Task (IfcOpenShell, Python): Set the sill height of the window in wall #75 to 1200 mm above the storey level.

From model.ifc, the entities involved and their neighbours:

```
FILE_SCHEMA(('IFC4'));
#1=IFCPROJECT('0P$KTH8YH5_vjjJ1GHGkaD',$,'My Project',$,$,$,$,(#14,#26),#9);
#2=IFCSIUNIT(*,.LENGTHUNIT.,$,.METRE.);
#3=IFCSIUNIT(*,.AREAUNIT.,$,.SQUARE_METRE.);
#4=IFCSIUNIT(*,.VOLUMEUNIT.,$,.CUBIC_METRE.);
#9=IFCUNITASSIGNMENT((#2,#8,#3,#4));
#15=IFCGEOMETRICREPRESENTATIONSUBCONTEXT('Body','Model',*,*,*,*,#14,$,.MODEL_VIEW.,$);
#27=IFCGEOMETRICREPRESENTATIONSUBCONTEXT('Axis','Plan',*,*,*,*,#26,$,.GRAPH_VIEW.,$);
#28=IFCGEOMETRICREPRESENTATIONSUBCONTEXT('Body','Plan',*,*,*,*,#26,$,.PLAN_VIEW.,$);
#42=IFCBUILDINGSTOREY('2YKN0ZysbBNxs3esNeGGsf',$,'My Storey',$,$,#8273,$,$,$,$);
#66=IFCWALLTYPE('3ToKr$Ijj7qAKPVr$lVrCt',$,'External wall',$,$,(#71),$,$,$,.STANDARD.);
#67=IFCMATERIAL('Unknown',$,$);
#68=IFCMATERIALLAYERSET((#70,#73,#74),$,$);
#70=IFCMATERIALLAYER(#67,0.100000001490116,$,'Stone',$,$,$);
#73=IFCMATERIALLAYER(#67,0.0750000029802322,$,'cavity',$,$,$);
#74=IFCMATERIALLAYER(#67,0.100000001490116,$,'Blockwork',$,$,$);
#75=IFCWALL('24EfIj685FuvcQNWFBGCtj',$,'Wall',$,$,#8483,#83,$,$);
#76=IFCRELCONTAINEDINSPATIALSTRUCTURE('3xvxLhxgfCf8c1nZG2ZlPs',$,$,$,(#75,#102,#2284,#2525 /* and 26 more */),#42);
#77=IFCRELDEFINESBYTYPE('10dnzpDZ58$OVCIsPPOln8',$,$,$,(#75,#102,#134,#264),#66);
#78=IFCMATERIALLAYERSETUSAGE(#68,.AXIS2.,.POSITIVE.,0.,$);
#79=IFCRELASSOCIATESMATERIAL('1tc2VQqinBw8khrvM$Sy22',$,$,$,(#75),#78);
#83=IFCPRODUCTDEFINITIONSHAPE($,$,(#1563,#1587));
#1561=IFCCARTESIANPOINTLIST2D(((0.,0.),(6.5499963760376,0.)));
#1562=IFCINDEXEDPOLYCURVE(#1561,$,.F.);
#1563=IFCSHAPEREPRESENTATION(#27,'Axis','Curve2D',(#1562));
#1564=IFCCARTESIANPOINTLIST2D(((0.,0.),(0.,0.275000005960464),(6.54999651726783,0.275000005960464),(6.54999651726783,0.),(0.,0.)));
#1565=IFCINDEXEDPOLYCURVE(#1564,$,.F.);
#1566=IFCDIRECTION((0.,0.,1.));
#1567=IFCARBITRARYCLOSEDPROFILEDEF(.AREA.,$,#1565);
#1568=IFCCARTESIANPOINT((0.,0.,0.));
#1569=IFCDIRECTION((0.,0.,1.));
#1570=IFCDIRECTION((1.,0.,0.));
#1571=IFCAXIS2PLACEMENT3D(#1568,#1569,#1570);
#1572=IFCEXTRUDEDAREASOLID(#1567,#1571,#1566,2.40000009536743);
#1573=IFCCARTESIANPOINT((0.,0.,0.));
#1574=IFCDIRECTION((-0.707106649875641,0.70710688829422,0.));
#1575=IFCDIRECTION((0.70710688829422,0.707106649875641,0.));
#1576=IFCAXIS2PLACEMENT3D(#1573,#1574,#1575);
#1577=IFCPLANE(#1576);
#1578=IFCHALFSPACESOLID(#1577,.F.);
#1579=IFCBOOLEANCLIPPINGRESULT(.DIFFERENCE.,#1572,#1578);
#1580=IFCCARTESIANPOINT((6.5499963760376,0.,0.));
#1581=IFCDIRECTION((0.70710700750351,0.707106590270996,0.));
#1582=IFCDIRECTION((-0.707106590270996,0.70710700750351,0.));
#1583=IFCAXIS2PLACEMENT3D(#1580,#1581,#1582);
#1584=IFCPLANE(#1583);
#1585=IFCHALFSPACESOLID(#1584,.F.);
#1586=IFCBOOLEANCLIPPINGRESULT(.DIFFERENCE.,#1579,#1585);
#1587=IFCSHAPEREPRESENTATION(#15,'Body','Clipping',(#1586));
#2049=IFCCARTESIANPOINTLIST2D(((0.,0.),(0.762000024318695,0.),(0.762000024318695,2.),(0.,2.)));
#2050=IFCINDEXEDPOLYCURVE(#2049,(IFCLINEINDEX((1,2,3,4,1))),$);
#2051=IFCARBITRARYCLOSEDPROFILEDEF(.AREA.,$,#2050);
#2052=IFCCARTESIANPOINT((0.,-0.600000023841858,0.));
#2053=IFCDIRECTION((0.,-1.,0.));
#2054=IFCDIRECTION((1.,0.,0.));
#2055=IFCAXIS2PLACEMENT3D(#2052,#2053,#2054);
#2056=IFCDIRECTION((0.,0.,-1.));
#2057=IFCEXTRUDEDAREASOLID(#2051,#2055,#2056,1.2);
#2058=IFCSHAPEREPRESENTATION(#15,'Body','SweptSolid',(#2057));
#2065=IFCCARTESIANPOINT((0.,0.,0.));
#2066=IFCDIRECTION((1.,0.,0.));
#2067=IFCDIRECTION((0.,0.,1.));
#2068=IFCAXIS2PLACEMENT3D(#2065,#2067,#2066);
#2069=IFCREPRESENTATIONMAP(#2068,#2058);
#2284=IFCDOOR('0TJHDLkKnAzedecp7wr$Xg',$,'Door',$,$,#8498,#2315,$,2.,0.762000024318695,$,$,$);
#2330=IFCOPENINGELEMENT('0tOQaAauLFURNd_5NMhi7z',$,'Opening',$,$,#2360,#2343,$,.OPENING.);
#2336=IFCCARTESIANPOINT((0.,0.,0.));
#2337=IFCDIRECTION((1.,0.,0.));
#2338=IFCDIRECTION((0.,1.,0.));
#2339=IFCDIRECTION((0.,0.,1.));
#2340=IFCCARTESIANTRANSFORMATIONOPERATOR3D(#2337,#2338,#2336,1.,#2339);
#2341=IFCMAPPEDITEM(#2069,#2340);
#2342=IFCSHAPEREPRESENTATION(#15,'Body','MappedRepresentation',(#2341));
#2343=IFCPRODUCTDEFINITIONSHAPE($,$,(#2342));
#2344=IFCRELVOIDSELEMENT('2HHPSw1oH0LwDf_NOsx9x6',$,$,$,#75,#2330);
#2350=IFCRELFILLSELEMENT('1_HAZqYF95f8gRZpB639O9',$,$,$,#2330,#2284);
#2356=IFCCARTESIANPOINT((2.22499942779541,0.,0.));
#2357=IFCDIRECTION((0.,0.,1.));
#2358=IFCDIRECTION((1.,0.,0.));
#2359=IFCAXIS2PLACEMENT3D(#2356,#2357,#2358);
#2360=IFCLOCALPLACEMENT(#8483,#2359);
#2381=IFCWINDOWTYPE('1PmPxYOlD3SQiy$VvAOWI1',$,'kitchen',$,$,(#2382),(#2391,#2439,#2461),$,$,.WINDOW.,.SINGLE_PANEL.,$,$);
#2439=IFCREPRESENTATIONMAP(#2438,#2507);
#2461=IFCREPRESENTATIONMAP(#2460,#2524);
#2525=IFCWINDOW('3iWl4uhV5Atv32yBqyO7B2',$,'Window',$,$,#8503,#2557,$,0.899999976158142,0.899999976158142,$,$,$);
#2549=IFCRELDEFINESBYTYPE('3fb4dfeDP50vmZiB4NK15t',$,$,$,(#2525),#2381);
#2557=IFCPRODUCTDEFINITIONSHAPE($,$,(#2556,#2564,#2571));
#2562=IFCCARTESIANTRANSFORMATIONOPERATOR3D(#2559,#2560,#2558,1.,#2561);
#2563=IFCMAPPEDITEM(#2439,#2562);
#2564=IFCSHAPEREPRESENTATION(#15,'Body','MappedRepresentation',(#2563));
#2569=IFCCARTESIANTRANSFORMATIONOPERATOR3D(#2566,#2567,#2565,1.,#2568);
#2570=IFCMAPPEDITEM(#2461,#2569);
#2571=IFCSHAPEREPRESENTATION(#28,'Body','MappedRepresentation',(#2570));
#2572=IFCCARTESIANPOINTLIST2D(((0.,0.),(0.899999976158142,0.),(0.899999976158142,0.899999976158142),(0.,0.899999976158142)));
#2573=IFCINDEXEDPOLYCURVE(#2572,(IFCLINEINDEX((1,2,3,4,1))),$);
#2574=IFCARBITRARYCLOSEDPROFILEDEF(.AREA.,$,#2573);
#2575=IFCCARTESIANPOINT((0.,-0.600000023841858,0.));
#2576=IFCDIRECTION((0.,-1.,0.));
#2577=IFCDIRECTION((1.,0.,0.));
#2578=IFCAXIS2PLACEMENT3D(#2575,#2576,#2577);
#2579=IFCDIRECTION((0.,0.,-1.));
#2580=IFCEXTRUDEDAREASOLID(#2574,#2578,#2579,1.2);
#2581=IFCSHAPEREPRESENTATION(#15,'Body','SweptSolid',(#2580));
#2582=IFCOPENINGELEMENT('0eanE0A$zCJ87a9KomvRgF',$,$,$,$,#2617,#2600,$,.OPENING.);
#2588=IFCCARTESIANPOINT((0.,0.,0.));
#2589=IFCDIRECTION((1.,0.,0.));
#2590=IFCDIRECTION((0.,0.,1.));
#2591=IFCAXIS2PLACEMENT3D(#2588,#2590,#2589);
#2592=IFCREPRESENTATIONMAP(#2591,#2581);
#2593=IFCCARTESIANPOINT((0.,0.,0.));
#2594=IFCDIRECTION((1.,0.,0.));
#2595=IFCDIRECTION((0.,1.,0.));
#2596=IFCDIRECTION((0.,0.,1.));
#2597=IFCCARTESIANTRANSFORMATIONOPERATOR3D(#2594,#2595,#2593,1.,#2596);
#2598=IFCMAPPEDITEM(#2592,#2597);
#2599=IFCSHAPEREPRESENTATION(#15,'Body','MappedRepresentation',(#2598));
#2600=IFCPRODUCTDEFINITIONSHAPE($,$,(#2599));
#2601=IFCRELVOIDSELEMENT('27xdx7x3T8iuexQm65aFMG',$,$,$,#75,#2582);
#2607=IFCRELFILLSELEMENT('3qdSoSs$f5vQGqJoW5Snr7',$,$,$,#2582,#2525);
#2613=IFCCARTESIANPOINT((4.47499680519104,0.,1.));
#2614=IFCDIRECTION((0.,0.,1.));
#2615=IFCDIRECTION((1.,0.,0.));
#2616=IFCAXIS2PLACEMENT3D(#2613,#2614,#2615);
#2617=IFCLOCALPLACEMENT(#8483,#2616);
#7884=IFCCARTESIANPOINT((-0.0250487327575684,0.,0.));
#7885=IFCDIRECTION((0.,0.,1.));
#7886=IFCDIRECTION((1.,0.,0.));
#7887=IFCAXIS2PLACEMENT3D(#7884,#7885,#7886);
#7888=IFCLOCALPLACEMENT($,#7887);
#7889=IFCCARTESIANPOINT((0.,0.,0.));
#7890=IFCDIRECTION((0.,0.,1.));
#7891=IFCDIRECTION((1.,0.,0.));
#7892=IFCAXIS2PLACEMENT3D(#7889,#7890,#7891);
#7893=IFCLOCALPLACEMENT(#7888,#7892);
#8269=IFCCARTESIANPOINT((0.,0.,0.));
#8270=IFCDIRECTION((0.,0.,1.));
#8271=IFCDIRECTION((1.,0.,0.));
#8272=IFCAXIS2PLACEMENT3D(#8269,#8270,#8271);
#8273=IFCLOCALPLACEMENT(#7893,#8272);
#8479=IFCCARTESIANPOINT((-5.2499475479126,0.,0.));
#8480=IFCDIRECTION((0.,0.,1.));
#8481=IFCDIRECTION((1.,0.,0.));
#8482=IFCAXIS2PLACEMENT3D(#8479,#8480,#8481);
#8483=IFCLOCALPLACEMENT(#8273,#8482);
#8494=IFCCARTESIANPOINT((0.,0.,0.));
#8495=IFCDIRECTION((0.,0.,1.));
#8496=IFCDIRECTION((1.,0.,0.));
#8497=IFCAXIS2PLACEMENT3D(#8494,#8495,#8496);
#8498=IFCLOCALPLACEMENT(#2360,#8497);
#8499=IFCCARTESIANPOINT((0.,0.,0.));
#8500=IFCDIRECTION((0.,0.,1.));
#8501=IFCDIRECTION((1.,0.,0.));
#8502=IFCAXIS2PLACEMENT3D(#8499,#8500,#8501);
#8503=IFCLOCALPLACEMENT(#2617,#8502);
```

```python
import numpy as np
import ifcopenshell
import ifcopenshell.api.geometry
import ifcopenshell.geom
import ifcopenshell.util.element
import ifcopenshell.util.placement
import ifcopenshell.util.shape
import ifcopenshell.util.unit

model = ifcopenshell.open("model.ifc")
unit_scale = ifcopenshell.util.unit.calculate_unit_scale(model)

window = model.by_guid("3iWl4uhV5Atv32yBqyO7B2")
opening = window.FillsVoids[0].RelatingOpeningElement
storey = ifcopenshell.util.element.get_container(window, ifc_class="IfcBuildingStorey")
level = ifcopenshell.util.placement.get_local_placement(storey.ObjectPlacement)[2, 3]

# The opening's origin need not be at the sill, so measure its lowest point.
shape = ifcopenshell.geom.create_shape(ifcopenshell.geom.settings(), opening)
bottom = ifcopenshell.util.shape.get_shape_bottom_elevation(shape, shape.geometry) / unit_scale
dz = level + 1.2 / unit_scale - bottom

shift = np.array([0.0, 0.0, dz])
# The window is placed relative to its opening, so it follows when the opening moves.
matrix = ifcopenshell.util.placement.get_local_placement(opening.ObjectPlacement)
matrix[:3, 3] += shift
ifcopenshell.api.geometry.edit_object_placement(
    model, product=opening, matrix=matrix, is_si=False, should_transform_children=True
)

print(f"moved by {dz * unit_scale:+.3f} m")

model.write("model_rev.ifc")
```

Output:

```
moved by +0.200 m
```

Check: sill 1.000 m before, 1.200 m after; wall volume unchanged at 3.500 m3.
